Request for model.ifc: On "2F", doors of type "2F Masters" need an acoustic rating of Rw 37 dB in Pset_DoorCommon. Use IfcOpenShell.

First a look at what the model holds.

```python
import ifcopenshell
import ifcopenshell.util.element

model = ifcopenshell.open("model.ifc")
print(model.schema)
storey = next(s for s in model.by_type("IfcBuildingStorey") if s.Name == "2F")
doors = [e for e in ifcopenshell.util.element.get_decomposition(storey) if e.is_a("IfcDoor")]
seen = {}
for e in doors:
    element_type = ifcopenshell.util.element.get_type(e)
    key = (element_type.Name if element_type != e and element_type else None, ifcopenshell.util.element.get_pset(e, "Pset_DoorCommon", "AcousticRating"))
    seen[key] = seen.get(key, 0) + 1
for (name, value), count in sorted(seen.items(), key=str):
    print(count, "x", name, "|", value)
```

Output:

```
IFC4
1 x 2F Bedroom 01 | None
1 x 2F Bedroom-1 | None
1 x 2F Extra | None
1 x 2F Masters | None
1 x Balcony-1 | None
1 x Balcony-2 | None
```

```python
import ifcopenshell
import ifcopenshell.api.pset
import ifcopenshell.util.element

model = ifcopenshell.open("model.ifc")

storey = next(s for s in model.by_type("IfcBuildingStorey") if s.Name == "2F")
doors = [e for e in ifcopenshell.util.element.get_decomposition(storey) if e.is_a("IfcDoor")]

count = 0
for e in doors:
    element_type = ifcopenshell.util.element.get_type(e)
    if element_type in (None, e) or element_type.Name != "2F Masters":
        continue
    # add_pset returns the element's existing set when there is one.
    pset = ifcopenshell.api.pset.add_pset(model, product=e, name="Pset_DoorCommon")
    ifcopenshell.api.pset.edit_pset(model, pset=pset, properties={"AcousticRating": "Rw 37 dB"})
    count += 1

print(count, "doors updated")

model.write("model_v2.ifc")
```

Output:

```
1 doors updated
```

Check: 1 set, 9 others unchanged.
